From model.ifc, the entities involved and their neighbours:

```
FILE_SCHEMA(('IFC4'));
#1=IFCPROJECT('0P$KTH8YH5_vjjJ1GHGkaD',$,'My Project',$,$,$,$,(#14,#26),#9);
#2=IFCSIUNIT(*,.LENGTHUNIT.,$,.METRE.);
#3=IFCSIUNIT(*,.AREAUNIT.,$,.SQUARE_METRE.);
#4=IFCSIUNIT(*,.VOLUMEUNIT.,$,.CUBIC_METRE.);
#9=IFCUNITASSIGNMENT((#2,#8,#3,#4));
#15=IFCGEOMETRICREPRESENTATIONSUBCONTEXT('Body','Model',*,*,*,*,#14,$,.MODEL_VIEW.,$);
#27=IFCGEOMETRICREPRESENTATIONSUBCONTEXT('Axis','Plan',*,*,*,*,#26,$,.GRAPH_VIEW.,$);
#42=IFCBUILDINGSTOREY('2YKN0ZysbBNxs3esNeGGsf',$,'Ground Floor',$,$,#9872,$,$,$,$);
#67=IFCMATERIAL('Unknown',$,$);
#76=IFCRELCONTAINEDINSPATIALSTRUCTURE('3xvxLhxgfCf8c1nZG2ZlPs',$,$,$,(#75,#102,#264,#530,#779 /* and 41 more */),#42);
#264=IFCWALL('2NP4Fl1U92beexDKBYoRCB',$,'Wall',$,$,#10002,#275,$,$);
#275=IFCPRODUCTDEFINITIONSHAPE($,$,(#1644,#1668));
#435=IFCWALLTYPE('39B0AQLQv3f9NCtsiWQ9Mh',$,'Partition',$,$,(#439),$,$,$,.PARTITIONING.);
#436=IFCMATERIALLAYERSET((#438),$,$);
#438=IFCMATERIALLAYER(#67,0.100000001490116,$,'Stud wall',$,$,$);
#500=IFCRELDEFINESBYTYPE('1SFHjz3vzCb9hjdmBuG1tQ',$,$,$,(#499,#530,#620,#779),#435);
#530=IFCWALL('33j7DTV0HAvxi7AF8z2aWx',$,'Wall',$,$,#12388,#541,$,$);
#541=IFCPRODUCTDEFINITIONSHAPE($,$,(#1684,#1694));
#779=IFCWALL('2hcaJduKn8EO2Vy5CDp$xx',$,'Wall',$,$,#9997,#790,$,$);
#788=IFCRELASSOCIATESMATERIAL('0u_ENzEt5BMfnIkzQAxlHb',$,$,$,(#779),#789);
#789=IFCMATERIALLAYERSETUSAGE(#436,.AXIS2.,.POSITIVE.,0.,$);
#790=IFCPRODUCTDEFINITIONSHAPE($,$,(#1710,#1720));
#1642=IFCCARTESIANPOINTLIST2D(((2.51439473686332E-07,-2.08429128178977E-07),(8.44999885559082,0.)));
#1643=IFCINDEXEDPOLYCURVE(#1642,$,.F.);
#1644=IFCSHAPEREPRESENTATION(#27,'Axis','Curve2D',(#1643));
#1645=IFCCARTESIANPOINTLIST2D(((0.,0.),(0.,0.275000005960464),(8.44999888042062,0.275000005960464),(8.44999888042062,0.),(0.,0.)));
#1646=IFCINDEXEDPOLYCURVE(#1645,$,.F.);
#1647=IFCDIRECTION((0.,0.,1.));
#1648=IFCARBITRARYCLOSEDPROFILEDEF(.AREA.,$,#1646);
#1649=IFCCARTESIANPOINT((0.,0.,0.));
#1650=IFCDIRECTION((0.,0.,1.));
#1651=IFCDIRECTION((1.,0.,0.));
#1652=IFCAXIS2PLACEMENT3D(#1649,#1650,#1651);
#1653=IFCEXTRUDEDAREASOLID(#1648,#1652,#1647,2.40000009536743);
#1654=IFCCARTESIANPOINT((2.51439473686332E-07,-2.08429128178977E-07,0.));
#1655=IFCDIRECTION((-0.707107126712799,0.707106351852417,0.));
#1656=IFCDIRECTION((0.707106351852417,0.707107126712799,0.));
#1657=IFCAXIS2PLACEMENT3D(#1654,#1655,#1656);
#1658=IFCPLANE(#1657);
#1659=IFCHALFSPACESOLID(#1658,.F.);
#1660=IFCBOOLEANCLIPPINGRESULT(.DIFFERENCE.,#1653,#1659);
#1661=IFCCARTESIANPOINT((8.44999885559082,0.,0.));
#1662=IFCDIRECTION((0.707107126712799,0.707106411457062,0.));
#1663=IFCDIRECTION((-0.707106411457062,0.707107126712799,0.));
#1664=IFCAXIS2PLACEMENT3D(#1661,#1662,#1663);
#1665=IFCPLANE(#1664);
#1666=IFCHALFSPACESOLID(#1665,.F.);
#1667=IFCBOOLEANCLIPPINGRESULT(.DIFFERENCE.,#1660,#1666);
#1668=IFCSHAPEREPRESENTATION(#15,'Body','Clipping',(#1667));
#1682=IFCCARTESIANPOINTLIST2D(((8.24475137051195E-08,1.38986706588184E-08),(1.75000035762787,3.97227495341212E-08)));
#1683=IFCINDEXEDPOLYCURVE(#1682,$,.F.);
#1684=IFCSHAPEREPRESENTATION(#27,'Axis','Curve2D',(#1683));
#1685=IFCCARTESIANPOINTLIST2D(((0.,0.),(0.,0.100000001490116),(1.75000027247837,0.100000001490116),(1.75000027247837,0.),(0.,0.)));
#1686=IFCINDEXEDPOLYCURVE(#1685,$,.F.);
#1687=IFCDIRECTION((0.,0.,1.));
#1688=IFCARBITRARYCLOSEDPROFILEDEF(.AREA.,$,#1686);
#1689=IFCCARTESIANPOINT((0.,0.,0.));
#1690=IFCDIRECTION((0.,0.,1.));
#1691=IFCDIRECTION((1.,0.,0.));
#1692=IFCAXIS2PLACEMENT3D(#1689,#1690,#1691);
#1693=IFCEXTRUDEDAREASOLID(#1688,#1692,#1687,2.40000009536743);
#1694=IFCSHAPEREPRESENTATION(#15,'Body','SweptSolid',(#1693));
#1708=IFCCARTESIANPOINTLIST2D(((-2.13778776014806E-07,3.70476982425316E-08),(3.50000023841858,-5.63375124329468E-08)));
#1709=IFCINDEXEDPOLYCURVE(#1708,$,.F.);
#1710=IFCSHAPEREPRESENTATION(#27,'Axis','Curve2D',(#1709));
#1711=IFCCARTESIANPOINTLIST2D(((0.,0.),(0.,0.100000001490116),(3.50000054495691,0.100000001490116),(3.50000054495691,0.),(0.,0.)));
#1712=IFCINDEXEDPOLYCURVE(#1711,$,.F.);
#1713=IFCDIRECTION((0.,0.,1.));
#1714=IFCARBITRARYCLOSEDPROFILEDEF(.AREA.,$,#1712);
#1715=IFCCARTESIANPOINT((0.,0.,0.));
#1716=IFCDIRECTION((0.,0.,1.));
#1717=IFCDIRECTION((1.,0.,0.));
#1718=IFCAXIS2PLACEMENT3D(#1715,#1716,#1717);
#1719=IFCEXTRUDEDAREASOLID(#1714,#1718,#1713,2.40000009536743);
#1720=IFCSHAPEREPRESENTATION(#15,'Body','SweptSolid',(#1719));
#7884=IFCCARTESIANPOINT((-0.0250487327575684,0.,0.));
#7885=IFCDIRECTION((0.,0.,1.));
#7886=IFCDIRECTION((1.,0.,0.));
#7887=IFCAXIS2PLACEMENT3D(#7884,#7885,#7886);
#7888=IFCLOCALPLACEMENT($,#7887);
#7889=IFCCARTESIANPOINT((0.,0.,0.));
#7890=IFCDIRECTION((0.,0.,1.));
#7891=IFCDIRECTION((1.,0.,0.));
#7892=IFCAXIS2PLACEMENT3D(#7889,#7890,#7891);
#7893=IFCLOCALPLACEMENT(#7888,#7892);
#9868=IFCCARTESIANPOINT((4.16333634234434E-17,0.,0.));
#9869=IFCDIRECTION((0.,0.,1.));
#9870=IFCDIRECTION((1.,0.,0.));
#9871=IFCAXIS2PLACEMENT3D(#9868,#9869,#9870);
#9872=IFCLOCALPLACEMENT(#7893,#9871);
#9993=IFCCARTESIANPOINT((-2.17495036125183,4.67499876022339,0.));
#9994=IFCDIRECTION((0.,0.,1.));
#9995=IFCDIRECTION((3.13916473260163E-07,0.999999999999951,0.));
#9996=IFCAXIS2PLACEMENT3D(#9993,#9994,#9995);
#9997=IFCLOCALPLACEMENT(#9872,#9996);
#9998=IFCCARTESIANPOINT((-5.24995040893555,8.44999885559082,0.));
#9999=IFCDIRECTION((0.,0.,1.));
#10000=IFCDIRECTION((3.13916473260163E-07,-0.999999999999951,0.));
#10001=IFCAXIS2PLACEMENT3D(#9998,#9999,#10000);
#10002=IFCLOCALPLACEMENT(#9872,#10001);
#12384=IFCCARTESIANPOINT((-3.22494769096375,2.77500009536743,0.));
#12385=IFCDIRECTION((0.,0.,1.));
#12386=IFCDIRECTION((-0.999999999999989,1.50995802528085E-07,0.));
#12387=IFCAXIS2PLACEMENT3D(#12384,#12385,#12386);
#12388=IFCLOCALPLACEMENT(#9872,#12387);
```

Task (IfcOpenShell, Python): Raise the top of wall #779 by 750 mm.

```python
import ifcopenshell
import ifcopenshell.geom
import ifcopenshell.util.representation
import ifcopenshell.util.shape
import ifcopenshell.util.unit

model = ifcopenshell.open("model.ifc")
unit_scale = ifcopenshell.util.unit.calculate_unit_scale(model)
settings = ifcopenshell.geom.settings()


def volume(element):
    """Net volume in cubic metres, openings subtracted."""
    shape = ifcopenshell.geom.create_shape(settings, element)
    return ifcopenshell.util.shape.get_volume(shape.geometry)


wall = model.by_id(779)
before = volume(wall)

body = ifcopenshell.util.representation.get_representation(wall, "Model", "Body")
solid = body.Items[0]
old_height = solid.Depth
solid.Depth += 0.75 / unit_scale
after = volume(wall)

print(f"height {old_height:g} -> {solid.Depth:g}, volume {before:.3f} -> {after:.3f} m3")

model.write("model_v2.ifc")
```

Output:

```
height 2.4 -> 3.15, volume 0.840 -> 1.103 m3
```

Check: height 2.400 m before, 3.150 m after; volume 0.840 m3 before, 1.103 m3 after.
